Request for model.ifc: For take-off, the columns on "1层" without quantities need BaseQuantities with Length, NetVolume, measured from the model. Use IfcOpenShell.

First a look at what the model holds.

```python
import ifcopenshell
import ifcopenshell.util.element
import ifcopenshell.util.unit

model = ifcopenshell.open("model.ifc")
print(model.schema)
for unit_type in ("LENGTHUNIT", "AREAUNIT", "VOLUMEUNIT"):
    print(unit_type, ifcopenshell.util.unit.calculate_unit_scale(model, unit_type))
storey = next(s for s in model.by_type("IfcBuildingStorey") if s.Name == "1层")
columns = [e for e in ifcopenshell.util.element.get_decomposition(storey) if e.is_a("IfcColumn")]
for e in sorted(columns, key=lambda e: e.id()):
    print(e.id(), e.is_a(), e.Name, list(ifcopenshell.util.element.get_psets(e, qtos_only=True)), sep=" | ")
```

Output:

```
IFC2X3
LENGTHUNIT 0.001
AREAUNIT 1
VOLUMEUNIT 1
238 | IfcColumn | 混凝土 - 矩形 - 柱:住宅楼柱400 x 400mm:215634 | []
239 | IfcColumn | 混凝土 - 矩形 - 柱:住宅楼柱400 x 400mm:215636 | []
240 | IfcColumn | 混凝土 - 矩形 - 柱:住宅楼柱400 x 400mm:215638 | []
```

```python
import ifcopenshell
import ifcopenshell.api.pset
import ifcopenshell.geom
import ifcopenshell.util.element
import ifcopenshell.util.shape
import ifcopenshell.util.unit

model = ifcopenshell.open("model.ifc")
unit_scale = ifcopenshell.util.unit.calculate_unit_scale(model)
volume_scale = ifcopenshell.util.unit.calculate_unit_scale(model, "VOLUMEUNIT")
settings = ifcopenshell.geom.settings()

storey = next(s for s in model.by_type("IfcBuildingStorey") if s.Name == "1层")
columns = [e for e in ifcopenshell.util.element.get_decomposition(storey) if e.is_a("IfcColumn")]

for e in sorted(columns, key=lambda e: e.id()):
    if ifcopenshell.util.element.get_psets(e, qtos_only=True, should_inherit=False):
        continue
    # Geometry comes back in metres, in the element's own axes.
    shape = ifcopenshell.geom.create_shape(settings, e)
    values = {
        "Length": ifcopenshell.util.shape.get_z(shape.geometry) / unit_scale,
        "NetVolume": ifcopenshell.util.shape.get_volume(shape.geometry) / volume_scale,
    }
    qto = ifcopenshell.api.pset.add_qto(model, product=e, name="BaseQuantities")
    ifcopenshell.api.pset.edit_qto(model, qto=qto, properties=values)
    print(e.id(), {k: round(v, 3) for k, v in values.items()})

model.write("model_edited.ifc")
```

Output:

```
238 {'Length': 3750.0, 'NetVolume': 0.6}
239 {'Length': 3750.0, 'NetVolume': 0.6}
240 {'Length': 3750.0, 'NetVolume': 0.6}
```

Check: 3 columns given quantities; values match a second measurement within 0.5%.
